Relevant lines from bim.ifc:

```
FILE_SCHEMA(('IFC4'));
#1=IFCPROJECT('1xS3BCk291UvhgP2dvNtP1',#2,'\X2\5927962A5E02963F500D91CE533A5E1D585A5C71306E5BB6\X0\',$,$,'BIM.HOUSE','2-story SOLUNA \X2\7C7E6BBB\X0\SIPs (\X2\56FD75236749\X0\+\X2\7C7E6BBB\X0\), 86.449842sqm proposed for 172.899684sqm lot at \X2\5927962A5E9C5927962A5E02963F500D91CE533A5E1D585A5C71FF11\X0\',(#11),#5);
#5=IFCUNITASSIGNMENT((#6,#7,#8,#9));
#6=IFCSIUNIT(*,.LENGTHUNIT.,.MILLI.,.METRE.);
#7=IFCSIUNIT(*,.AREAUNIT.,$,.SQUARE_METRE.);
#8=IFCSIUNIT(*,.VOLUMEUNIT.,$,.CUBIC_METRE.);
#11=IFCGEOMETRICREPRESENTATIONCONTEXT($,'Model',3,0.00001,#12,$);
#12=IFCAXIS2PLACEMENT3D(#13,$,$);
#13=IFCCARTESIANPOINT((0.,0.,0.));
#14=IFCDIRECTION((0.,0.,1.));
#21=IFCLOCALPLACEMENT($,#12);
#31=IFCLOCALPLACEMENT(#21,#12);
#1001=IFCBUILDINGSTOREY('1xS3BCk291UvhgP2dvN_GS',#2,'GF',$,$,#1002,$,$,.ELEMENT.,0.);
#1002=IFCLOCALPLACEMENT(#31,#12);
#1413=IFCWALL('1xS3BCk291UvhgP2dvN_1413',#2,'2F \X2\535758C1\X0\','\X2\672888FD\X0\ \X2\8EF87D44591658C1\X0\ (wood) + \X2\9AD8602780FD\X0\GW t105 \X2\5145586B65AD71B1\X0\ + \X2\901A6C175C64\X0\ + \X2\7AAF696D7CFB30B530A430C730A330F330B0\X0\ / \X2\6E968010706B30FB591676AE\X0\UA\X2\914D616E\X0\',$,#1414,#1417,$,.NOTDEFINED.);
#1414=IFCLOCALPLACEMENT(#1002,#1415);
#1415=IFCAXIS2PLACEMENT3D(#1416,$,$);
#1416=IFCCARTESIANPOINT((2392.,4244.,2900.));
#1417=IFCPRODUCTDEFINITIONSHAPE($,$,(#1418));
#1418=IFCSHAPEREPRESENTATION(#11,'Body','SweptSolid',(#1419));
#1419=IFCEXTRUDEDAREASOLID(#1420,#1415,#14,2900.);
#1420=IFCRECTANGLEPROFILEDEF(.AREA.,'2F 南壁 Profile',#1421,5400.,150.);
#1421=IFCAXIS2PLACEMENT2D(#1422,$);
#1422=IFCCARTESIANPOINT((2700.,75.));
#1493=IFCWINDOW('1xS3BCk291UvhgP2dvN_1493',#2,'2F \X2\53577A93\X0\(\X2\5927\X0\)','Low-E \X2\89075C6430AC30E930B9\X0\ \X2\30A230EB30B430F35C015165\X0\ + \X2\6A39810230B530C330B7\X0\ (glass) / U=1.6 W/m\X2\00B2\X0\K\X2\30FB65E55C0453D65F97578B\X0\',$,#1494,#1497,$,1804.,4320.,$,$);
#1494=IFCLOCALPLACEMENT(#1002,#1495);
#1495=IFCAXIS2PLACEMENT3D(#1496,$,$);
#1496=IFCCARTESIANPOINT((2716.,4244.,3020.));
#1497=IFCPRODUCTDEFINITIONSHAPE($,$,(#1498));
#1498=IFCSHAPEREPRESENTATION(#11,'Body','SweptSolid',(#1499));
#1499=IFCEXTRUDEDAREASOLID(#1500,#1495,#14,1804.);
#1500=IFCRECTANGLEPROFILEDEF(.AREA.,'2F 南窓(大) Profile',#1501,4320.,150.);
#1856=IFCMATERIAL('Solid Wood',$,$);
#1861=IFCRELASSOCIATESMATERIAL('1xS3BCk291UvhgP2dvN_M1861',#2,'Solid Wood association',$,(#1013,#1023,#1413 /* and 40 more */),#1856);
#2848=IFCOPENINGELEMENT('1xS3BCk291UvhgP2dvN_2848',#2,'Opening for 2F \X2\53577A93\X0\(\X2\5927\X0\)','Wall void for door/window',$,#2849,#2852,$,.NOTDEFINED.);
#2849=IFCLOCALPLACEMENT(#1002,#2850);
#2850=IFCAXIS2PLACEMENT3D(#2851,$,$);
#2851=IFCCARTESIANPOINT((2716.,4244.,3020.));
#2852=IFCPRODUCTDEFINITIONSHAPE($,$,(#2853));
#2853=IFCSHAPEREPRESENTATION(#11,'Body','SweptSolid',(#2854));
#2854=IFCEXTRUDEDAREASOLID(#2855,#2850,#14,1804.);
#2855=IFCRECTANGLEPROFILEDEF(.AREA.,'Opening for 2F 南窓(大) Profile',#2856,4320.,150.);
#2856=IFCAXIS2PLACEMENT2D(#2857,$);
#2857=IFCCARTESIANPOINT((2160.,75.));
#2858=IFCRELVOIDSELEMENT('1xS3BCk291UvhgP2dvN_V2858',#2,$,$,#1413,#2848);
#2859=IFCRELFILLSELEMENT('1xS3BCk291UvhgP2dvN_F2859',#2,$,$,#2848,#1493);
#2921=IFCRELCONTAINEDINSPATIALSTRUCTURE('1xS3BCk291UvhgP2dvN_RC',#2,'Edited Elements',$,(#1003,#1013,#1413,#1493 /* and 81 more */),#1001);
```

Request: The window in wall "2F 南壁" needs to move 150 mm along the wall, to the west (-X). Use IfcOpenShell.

```python
import ifcopenshell
import ifcopenshell.api.geometry
import ifcopenshell.util.placement
import ifcopenshell.util.unit

model = ifcopenshell.open("bim.ifc")
unit_scale = ifcopenshell.util.unit.calculate_unit_scale(model)

window = model.by_id(1493)
opening = window.FillsVoids[0].RelatingOpeningElement
wall = opening.VoidsElements[0].RelatingBuildingElement

wall_matrix = ifcopenshell.util.placement.get_local_placement(wall.ObjectPlacement)
shift = wall_matrix[:3, 0] * -0.15 / unit_scale
before = ifcopenshell.util.placement.get_local_placement(window.ObjectPlacement)[:3, 3].copy()

# The window is not placed relative to its opening, so move both.
for product in (opening, window):
    matrix = ifcopenshell.util.placement.get_local_placement(product.ObjectPlacement)
    matrix[:3, 3] += shift
    ifcopenshell.api.geometry.edit_object_placement(model, product=product, matrix=matrix, is_si=False)

after = ifcopenshell.util.placement.get_local_placement(window.ObjectPlacement)[:3, 3]
print("window moved by", (after - before).round(3) + 0.0)

model.write("bim_updated.ifc")
```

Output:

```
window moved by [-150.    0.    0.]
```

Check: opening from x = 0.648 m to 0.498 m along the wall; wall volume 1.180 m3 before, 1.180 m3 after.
